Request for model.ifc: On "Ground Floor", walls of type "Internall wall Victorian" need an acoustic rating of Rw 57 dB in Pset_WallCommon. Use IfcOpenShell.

First a look at what the model holds.

```python
import ifcopenshell
import ifcopenshell.util.element

model = ifcopenshell.open("model.ifc")
print(model.schema)
storey = next(s for s in model.by_type("IfcBuildingStorey") if s.Name == "Ground Floor")
walls = [e for e in ifcopenshell.util.element.get_decomposition(storey) if e.is_a("IfcWall")]
seen = {}
for e in walls:
    element_type = ifcopenshell.util.element.get_type(e)
    key = (element_type.Name if element_type != e and element_type else None, ifcopenshell.util.element.get_pset(e, "Pset_WallCommon", "AcousticRating"))
    seen[key] = seen.get(key, 0) + 1
for (name, value), count in sorted(seen.items(), key=str):
    print(count, "x", name, "|", value)
```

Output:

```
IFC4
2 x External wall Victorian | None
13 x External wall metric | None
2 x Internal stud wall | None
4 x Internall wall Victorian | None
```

```python
import ifcopenshell
import ifcopenshell.api.pset
import ifcopenshell.util.element

model = ifcopenshell.open("model.ifc")

storey = next(s for s in model.by_type("IfcBuildingStorey") if s.Name == "Ground Floor")
walls = [e for e in ifcopenshell.util.element.get_decomposition(storey) if e.is_a("IfcWall")]

count = 0
for e in walls:
    element_type = ifcopenshell.util.element.get_type(e)
    if element_type in (None, e) or element_type.Name != "Internall wall Victorian":
        continue
    # add_pset returns the element's existing set when there is one.
    pset = ifcopenshell.api.pset.add_pset(model, product=e, name="Pset_WallCommon")
    ifcopenshell.api.pset.edit_pset(model, pset=pset, properties={"AcousticRating": "Rw 57 dB"})
    count += 1

print(count, "walls updated")

model.write("model_edited.ifc")
```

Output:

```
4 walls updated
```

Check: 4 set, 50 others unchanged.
